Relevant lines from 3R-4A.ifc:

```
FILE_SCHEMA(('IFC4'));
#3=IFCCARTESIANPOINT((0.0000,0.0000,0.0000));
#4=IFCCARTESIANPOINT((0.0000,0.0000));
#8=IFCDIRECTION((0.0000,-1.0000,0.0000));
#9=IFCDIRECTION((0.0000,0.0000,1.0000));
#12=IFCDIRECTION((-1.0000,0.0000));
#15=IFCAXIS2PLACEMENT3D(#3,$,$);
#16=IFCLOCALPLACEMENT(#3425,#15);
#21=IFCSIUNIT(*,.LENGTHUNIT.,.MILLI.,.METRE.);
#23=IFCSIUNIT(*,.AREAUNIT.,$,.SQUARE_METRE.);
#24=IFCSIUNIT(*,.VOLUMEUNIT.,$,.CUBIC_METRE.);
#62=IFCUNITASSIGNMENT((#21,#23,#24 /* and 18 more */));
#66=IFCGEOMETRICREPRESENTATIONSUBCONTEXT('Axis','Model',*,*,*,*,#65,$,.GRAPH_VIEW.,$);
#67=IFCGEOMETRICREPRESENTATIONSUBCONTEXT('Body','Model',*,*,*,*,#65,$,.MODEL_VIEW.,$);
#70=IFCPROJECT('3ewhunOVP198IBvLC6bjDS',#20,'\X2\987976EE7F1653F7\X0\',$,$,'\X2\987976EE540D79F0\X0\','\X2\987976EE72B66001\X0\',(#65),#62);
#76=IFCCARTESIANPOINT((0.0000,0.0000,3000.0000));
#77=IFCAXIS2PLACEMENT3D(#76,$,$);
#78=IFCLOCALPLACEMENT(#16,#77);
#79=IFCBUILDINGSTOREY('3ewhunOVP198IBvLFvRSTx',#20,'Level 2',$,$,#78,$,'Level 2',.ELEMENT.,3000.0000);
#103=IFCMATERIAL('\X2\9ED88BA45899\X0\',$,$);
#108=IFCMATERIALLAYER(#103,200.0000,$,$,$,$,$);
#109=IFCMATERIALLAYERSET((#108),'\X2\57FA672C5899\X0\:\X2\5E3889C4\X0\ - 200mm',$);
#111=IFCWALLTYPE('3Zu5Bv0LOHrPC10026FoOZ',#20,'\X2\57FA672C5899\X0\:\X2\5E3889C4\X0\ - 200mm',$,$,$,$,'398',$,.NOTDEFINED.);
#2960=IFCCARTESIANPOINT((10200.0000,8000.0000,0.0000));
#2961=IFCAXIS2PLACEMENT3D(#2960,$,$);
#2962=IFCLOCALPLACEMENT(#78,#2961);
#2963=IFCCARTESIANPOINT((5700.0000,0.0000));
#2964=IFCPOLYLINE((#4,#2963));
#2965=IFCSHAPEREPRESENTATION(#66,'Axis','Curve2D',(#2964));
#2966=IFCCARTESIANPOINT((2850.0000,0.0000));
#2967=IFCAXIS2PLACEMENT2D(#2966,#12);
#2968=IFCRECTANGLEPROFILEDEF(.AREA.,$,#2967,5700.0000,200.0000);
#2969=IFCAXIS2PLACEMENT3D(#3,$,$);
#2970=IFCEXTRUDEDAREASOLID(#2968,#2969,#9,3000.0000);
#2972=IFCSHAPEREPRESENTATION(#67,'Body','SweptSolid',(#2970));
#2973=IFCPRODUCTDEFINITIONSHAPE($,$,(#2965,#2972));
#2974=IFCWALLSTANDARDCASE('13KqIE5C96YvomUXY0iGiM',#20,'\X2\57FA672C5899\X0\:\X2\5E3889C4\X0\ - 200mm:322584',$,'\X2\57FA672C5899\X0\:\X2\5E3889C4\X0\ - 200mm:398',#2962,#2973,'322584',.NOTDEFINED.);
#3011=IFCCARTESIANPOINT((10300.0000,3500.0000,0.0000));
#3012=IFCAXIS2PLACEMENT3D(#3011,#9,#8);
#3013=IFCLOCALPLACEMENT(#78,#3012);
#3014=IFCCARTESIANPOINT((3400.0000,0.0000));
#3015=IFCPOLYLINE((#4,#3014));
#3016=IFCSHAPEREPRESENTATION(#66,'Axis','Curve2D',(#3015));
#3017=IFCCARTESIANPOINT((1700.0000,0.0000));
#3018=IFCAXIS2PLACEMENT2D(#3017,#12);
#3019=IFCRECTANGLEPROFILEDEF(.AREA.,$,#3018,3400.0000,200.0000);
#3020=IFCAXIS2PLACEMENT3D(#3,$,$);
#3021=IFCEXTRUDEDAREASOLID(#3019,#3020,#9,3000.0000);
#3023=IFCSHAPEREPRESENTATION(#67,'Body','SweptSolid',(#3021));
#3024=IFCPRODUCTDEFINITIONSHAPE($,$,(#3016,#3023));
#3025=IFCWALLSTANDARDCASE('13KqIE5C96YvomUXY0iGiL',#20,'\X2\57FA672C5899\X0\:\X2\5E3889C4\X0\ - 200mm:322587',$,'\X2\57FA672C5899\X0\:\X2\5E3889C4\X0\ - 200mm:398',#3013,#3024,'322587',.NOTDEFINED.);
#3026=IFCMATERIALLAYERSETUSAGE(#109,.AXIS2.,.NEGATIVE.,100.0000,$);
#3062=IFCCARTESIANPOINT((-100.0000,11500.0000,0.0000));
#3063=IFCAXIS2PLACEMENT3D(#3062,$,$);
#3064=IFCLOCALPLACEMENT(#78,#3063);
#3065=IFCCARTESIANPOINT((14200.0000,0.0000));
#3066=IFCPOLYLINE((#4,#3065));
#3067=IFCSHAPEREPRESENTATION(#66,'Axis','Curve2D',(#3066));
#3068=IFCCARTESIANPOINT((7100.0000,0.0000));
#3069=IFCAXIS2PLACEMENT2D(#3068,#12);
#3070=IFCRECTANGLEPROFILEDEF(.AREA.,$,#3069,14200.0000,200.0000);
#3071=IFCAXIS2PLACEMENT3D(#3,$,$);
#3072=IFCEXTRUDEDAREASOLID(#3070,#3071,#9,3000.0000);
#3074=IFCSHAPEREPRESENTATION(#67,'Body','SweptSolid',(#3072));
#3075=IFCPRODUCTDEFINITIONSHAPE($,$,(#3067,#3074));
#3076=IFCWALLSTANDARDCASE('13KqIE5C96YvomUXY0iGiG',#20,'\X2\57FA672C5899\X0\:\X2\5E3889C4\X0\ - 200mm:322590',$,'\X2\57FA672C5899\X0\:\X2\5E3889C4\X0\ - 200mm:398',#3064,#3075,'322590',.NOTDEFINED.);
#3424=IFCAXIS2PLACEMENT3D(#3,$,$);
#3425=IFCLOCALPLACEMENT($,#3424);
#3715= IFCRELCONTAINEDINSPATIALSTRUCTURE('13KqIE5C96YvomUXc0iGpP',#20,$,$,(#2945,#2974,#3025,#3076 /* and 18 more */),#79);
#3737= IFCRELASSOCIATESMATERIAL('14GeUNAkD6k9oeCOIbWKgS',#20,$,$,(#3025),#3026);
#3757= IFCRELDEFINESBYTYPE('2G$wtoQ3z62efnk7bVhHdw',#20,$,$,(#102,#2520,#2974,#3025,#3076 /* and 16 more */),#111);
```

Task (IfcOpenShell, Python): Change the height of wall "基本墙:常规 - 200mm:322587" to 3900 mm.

```python
import ifcopenshell
import ifcopenshell.geom
import ifcopenshell.util.representation
import ifcopenshell.util.shape

model = ifcopenshell.open("3R-4A.ifc")
settings = ifcopenshell.geom.settings()


def volume(element):
    """Net volume in cubic metres, openings subtracted."""
    shape = ifcopenshell.geom.create_shape(settings, element)
    return ifcopenshell.util.shape.get_volume(shape.geometry)


wall = model.by_guid("13KqIE5C96YvomUXY0iGiL")
before = volume(wall)

body = ifcopenshell.util.representation.get_representation(wall, "Model", "Body")
solid = body.Items[0]
old_height = solid.Depth
solid.Depth = 3900.0
after = volume(wall)

print(f"height {old_height:g} -> {solid.Depth:g}, volume {before:.3f} -> {after:.3f} m3")

model.write("3R-4A-out.ifc")
```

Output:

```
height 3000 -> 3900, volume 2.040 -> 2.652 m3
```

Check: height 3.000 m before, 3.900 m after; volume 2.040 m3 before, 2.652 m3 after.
